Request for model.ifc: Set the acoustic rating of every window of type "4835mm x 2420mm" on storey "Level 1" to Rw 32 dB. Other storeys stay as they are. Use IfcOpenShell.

First a look at what the model holds.

```python
import ifcopenshell
import ifcopenshell.util.element

model = ifcopenshell.open("model.ifc")
print(model.schema)
storey = next(s for s in model.by_type("IfcBuildingStorey") if s.Name == "Level 1")
windows = [e for e in ifcopenshell.util.element.get_decomposition(storey) if e.is_a("IfcWindow")]
seen = {}
for e in windows:
    element_type = ifcopenshell.util.element.get_type(e)
    key = (element_type.Name if element_type != e and element_type else None, ifcopenshell.util.element.get_pset(e, "Pset_WindowCommon", "AcousticRating"))
    seen[key] = seen.get(key, 0) + 1
for (name, value), count in sorted(seen.items(), key=str):
    print(count, "x", name, "|", value)
```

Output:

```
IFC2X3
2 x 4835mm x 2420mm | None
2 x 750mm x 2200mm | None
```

```python
import ifcopenshell
import ifcopenshell.api.pset
import ifcopenshell.util.element

model = ifcopenshell.open("model.ifc")

storey = next(s for s in model.by_type("IfcBuildingStorey") if s.Name == "Level 1")
windows = [e for e in ifcopenshell.util.element.get_decomposition(storey) if e.is_a("IfcWindow")]

count = 0
for e in windows:
    element_type = ifcopenshell.util.element.get_type(e)
    if element_type in (None, e) or element_type.Name != "4835mm x 2420mm":
        continue
    # add_pset returns the element's existing set when there is one.
    pset = ifcopenshell.api.pset.add_pset(model, product=e, name="Pset_WindowCommon")
    ifcopenshell.api.pset.edit_pset(model, pset=pset, properties={"AcousticRating": "Rw 32 dB"})
    count += 1

print(count, "windows updated")

model.write("model_edited.ifc")
```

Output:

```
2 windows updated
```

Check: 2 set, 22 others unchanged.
